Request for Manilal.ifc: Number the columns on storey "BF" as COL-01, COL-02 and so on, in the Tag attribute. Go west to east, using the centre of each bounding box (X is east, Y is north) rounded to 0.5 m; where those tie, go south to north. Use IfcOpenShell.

First a look at what the model holds.

```python
import ifcopenshell
import ifcopenshell.util.element
import ifcopenshell.util.placement

model = ifcopenshell.open("Manilal.ifc")
print(model.schema)
storey = next(s for s in model.by_type("IfcBuildingStorey") if s.Name == "BF")
columns = [e for e in ifcopenshell.util.element.get_decomposition(storey) if e.is_a("IfcColumn")]
for e in sorted(columns, key=lambda e: e.id()):
    origin = ifcopenshell.util.placement.get_local_placement(e.ObjectPlacement)[:3, 3]
    print(e.id(), e.Tag, e.Name, origin.round(2) + 0.0, sep=" | ")
```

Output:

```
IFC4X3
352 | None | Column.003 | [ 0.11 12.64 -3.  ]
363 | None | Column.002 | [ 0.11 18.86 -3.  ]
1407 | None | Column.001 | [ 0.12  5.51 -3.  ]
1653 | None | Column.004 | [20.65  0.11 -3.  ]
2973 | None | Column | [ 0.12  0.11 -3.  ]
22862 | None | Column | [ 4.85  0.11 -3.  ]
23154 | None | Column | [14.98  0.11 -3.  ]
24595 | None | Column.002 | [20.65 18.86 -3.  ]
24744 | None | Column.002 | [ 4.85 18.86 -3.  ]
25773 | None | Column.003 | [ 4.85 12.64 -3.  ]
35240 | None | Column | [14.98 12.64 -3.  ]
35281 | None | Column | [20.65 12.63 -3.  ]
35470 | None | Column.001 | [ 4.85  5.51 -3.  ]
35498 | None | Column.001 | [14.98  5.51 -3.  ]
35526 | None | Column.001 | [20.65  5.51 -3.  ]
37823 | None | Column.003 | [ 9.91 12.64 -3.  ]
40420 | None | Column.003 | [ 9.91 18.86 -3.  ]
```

```python
import ifcopenshell
import ifcopenshell.geom
import ifcopenshell.util.element
import ifcopenshell.util.shape

model = ifcopenshell.open("Manilal.ifc")
settings = ifcopenshell.geom.settings()
settings.set("use-world-coords", True)


def centre(element):
    shape = ifcopenshell.geom.create_shape(settings, element)
    return ifcopenshell.util.shape.get_bbox_centroid(shape.geometry)


storey = next(s for s in model.by_type("IfcBuildingStorey") if s.Name == "BF")
columns = [e for e in ifcopenshell.util.element.get_decomposition(storey) if e.is_a("IfcColumn")]

# Insertion points can sit at a corner or the storey origin, so sort by the geometry (in metres).
centres = {e: centre(e) for e in columns}
columns.sort(key=lambda e: (round(centres[e][0] / 0.5), centres[e][1]))

for i, e in enumerate(columns, start=1):
    number = f"COL-{i:02d}"
    e.Tag = number
    print(e.id(), number)

model.write("Manilal_edited.ifc")
```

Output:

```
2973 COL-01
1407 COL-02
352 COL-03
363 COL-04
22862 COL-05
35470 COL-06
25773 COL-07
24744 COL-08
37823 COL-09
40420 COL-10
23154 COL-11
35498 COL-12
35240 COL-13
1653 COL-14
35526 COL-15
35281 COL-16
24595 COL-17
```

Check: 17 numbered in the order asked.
